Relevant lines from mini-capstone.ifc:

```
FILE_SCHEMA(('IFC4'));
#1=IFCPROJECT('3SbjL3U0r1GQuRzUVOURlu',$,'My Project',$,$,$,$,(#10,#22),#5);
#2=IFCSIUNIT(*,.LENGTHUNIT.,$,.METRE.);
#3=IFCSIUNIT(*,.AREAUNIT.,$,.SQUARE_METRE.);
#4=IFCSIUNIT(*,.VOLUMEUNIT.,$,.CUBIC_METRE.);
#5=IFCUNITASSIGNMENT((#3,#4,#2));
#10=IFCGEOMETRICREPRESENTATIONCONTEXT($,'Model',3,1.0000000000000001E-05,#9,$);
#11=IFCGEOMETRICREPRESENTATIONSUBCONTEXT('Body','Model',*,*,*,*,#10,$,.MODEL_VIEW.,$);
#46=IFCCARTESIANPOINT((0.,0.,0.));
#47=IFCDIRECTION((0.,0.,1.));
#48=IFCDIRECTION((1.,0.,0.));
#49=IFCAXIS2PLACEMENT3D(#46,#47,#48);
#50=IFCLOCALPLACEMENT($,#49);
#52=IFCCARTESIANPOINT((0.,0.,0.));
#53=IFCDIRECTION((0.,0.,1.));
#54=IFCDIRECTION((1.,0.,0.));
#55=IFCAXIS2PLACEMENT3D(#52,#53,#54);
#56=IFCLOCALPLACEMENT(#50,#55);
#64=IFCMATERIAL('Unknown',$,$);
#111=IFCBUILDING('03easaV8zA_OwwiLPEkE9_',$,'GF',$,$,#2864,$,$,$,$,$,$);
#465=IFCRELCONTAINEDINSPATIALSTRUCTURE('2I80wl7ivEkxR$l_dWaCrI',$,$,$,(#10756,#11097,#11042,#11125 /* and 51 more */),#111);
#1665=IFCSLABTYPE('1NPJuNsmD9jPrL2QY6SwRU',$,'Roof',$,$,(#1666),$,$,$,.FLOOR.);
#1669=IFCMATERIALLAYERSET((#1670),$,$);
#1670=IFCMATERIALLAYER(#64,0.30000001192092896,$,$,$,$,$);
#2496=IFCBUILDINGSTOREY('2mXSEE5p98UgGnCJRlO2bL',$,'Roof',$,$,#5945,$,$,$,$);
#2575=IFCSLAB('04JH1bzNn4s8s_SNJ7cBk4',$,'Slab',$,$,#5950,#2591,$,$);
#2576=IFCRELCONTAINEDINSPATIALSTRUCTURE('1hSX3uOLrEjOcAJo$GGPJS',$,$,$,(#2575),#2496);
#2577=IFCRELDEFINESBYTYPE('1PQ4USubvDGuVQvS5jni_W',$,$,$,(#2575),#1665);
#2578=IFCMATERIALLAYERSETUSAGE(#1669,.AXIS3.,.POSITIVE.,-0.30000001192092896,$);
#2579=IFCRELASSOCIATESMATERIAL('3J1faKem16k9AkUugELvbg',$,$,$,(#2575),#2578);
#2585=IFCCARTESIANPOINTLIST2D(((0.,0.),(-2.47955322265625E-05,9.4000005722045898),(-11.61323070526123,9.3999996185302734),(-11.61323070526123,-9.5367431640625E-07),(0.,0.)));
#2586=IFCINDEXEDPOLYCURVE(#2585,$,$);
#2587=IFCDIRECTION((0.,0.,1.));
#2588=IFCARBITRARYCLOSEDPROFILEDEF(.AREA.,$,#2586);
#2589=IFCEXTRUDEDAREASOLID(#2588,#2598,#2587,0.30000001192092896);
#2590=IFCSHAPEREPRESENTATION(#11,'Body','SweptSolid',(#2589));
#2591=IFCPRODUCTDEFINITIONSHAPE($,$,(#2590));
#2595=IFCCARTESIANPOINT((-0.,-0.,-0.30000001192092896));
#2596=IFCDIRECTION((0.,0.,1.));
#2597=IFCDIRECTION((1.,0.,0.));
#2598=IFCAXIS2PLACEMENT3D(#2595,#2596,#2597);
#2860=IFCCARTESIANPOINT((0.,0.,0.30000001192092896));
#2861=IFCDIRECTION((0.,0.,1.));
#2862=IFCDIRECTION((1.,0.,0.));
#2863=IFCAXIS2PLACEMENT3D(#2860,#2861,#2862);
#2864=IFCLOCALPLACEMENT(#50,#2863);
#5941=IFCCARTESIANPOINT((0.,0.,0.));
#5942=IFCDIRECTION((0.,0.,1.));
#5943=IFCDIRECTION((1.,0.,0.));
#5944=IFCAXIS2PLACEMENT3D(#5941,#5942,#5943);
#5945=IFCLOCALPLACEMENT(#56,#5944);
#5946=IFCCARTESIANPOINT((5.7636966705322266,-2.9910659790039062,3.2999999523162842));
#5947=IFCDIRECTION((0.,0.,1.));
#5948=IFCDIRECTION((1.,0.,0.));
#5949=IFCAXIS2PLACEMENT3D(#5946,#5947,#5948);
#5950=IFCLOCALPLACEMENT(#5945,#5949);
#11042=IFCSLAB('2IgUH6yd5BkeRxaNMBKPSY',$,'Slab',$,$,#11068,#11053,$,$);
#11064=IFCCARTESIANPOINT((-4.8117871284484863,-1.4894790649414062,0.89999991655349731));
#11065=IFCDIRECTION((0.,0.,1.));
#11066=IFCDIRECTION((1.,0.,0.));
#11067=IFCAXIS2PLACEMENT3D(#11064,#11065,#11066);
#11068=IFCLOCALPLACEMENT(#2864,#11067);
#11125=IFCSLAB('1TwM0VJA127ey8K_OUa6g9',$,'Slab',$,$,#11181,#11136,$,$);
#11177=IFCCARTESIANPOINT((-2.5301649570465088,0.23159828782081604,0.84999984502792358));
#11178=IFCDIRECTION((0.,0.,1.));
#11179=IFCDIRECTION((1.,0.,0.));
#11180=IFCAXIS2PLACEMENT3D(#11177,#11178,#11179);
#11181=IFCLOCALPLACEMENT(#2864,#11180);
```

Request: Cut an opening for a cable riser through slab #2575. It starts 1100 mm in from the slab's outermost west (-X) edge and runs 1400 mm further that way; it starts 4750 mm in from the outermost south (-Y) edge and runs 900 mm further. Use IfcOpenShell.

```python
import numpy as np
import ifcopenshell
import ifcopenshell.api.feature
import ifcopenshell.api.geometry
import ifcopenshell.api.root
import ifcopenshell.geom
import ifcopenshell.util.placement
import ifcopenshell.util.representation
import ifcopenshell.util.shape
import ifcopenshell.util.unit

model = ifcopenshell.open("mini-capstone.ifc")
unit_scale = ifcopenshell.util.unit.calculate_unit_scale(model)
settings = ifcopenshell.geom.settings()


def volume(element):
    """Net volume in cubic metres, openings subtracted."""
    shape = ifcopenshell.geom.create_shape(settings, element)
    return ifcopenshell.util.shape.get_volume(shape.geometry)


slab = model.by_id(2575)
before = volume(slab)

# Extent in the slab's own axes, in metres. The edges named are its -X and -Y sides.
slab_shape = ifcopenshell.geom.create_shape(settings, slab)
vertices = ifcopenshell.util.shape.get_vertices(slab_shape.geometry)
x_min, y_min, bottom = vertices.min(axis=0)
top = vertices[:, 2].max()

opening = ifcopenshell.api.root.create_entity(model, ifc_class="IfcOpeningElement", name="Cable riser opening", predefined_type="OPENING")
context = ifcopenshell.util.representation.get_context(model, "Model", "Body", "MODEL_VIEW")
width, depth = 1.4, 0.9
outline = [(0.0, 0.0), (width, 0.0), (width, depth), (0.0, depth), (0.0, 0.0)]
# Overshoot both faces by 50 mm so the cut is clean.
shape = ifcopenshell.api.geometry.add_slab_representation(
    model, context=context, depth=top - bottom + 0.1, polyline=outline
)
ifcopenshell.api.geometry.assign_representation(model, product=opening, representation=shape)

matrix = ifcopenshell.util.placement.get_local_placement(slab.ObjectPlacement)
matrix[:, 3] = matrix @ np.append(np.array([x_min + 1.1, y_min + 4.75, bottom - 0.05]) / unit_scale, 1.0)
ifcopenshell.api.geometry.edit_object_placement(model, product=opening, matrix=matrix, is_si=False)
ifcopenshell.api.feature.add_feature(model, feature=opening, element=slab)

after = volume(slab)

print(f"slab volume {before:.3f} -> {after:.3f} m3")

model.write("mini-capstone_edited.ifc")
```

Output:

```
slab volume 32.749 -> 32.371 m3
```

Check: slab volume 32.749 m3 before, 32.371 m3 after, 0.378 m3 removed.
